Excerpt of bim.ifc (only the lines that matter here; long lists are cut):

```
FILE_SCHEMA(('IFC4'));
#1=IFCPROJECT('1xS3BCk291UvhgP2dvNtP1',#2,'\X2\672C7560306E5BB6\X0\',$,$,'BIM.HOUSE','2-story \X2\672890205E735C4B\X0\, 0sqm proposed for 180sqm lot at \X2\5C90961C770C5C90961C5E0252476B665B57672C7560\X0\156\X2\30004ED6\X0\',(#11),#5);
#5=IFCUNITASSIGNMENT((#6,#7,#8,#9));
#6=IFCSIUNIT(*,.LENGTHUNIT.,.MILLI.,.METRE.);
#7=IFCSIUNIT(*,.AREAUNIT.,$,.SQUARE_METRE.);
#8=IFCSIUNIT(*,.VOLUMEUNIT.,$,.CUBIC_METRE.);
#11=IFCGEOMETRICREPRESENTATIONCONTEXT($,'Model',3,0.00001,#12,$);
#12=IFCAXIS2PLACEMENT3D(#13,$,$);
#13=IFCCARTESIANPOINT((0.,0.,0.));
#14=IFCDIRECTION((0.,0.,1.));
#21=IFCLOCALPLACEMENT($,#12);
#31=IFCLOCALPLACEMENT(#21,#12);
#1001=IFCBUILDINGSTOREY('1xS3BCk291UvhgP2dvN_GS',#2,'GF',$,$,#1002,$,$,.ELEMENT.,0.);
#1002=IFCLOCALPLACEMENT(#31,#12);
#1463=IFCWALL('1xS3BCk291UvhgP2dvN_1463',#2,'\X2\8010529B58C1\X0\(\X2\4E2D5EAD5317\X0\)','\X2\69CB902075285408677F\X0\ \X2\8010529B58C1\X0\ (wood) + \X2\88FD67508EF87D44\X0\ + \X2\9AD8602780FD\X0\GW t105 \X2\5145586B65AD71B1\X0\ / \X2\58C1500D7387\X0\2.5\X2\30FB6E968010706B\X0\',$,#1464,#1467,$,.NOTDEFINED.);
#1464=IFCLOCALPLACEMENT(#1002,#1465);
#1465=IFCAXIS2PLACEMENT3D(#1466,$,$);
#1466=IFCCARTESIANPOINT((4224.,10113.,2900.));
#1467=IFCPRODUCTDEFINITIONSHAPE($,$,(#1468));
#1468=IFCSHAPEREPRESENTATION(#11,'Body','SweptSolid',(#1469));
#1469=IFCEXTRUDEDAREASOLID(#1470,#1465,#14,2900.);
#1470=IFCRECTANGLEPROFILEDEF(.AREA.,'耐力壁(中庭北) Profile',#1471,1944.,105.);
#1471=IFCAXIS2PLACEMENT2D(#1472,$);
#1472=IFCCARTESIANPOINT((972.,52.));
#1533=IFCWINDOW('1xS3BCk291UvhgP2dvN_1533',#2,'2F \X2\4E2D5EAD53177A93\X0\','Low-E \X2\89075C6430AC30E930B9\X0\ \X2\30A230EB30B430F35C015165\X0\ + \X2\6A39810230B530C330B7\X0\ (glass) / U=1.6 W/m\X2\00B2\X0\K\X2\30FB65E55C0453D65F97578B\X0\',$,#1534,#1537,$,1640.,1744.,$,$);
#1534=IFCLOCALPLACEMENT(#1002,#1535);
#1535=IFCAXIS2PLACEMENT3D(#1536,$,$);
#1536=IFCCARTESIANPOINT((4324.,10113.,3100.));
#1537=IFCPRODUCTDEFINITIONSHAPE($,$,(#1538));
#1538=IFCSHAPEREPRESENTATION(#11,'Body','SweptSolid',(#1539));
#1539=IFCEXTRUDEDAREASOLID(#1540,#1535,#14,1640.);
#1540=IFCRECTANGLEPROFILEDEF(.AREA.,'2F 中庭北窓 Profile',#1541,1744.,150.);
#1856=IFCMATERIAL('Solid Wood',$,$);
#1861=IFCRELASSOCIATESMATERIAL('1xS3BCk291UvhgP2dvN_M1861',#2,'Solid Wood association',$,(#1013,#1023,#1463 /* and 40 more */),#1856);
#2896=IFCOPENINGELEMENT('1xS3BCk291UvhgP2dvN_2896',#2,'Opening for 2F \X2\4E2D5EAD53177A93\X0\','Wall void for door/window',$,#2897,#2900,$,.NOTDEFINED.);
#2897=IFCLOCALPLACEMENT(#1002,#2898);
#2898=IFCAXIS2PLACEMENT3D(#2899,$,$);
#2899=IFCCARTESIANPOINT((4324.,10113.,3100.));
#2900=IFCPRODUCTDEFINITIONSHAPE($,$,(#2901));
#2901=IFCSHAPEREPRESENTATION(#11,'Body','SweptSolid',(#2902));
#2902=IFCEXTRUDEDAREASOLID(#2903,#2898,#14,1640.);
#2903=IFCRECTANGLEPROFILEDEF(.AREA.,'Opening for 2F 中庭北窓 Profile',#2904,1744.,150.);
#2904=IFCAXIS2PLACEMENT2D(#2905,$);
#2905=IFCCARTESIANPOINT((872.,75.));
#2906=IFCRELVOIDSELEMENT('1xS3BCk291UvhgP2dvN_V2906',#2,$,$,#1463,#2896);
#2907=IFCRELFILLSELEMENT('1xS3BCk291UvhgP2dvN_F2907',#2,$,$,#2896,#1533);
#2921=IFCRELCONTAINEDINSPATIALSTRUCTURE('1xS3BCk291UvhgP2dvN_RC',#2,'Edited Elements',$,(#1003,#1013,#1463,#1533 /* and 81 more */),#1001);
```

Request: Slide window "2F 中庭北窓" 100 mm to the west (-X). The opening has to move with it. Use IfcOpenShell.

```python
import ifcopenshell
import ifcopenshell.api.geometry
import ifcopenshell.util.placement

model = ifcopenshell.open("bim.ifc")

window = model.by_guid("1xS3BCk291UvhgP2dvN_1533")
opening = window.FillsVoids[0].RelatingOpeningElement
wall = opening.VoidsElements[0].RelatingBuildingElement

wall_matrix = ifcopenshell.util.placement.get_local_placement(wall.ObjectPlacement)
shift = wall_matrix[:3, 0] * -100.0
before = ifcopenshell.util.placement.get_local_placement(window.ObjectPlacement)[:3, 3].copy()

# The window is not placed relative to its opening, so move both.
for product in (opening, window):
    matrix = ifcopenshell.util.placement.get_local_placement(product.ObjectPlacement)
    matrix[:3, 3] += shift
    ifcopenshell.api.geometry.edit_object_placement(model, product=product, matrix=matrix, is_si=False)

after = ifcopenshell.util.placement.get_local_placement(window.ObjectPlacement)[:3, 3]
print("window moved by", (after - before).round(3) + 0.0)

model.write("bim_updated.ifc")
```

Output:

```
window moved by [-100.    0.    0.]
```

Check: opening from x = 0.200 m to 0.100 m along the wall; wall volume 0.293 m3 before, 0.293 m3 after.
